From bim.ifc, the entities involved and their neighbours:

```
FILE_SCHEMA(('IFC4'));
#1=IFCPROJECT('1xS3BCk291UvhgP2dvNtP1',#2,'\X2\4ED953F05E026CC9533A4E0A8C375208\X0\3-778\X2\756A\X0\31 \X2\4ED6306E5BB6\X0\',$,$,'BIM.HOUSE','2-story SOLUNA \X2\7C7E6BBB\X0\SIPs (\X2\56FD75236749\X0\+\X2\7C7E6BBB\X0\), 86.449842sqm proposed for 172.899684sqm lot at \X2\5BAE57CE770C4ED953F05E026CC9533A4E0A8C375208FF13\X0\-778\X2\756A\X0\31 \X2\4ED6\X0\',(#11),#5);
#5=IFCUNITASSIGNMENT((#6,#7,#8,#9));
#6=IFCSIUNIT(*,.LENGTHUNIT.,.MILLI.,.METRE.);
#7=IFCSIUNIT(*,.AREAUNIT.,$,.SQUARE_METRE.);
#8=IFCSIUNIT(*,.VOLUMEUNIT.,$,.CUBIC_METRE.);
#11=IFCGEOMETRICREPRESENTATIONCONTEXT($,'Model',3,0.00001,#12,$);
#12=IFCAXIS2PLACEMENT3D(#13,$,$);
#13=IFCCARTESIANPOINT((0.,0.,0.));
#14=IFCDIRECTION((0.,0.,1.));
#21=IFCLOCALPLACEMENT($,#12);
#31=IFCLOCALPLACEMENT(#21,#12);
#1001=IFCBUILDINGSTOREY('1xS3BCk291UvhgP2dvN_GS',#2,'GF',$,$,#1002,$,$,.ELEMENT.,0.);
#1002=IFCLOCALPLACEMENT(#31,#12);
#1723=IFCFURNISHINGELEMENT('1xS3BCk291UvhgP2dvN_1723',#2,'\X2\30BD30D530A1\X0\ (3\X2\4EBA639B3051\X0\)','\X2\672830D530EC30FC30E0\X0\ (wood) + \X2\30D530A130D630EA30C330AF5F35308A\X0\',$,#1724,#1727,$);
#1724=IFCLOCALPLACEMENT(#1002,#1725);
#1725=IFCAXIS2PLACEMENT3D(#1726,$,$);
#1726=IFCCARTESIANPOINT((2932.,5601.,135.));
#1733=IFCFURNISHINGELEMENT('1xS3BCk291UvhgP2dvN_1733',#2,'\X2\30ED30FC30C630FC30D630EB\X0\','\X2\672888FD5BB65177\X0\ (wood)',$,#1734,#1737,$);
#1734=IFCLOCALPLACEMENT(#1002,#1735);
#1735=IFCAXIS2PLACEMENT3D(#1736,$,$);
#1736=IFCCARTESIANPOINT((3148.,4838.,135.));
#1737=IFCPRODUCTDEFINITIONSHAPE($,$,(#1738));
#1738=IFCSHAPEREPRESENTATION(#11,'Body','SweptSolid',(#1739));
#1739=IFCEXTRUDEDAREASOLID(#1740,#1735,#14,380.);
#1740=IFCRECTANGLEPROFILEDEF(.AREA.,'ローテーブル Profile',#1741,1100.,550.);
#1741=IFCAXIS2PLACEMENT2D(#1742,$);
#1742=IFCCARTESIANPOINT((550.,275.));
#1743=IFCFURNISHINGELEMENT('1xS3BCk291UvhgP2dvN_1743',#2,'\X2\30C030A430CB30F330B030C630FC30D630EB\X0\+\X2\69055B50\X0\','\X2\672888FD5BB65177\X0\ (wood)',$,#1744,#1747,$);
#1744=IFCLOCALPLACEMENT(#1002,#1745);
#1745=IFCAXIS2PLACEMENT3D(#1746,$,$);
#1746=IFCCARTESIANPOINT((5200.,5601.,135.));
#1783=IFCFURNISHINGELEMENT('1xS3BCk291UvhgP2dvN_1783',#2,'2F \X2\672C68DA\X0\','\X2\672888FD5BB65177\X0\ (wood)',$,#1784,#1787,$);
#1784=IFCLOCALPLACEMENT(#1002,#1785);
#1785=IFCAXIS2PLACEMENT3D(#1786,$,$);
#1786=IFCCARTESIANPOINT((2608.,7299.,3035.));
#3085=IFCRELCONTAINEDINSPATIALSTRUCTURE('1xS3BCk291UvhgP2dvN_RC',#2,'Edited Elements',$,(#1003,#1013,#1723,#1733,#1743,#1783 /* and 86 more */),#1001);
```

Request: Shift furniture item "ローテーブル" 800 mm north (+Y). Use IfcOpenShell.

```python
import ifcopenshell
import ifcopenshell.api.geometry
import ifcopenshell.util.placement

model = ifcopenshell.open("bim.ifc")

item = model.by_id(1733)
matrix = ifcopenshell.util.placement.get_local_placement(item.ObjectPlacement)
matrix[1, 3] += 800.0
ifcopenshell.api.geometry.edit_object_placement(model, product=item, matrix=matrix, is_si=False)

print(ifcopenshell.util.placement.get_local_placement(item.ObjectPlacement).round(3) + 0.0)

model.write("bim_edited.ifc")
```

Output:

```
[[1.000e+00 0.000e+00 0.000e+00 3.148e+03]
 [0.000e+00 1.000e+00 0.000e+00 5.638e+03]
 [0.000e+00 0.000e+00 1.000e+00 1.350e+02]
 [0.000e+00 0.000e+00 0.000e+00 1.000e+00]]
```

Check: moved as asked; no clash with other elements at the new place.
